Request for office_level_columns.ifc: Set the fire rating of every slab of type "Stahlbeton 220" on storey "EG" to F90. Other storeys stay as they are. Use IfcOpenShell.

First a look at what the model holds.

```python
import ifcopenshell
import ifcopenshell.util.element

model = ifcopenshell.open("office_level_columns.ifc")
print(model.schema)
storey = next(s for s in model.by_type("IfcBuildingStorey") if s.Name == "EG")
slabs = [e for e in ifcopenshell.util.element.get_decomposition(storey) if e.is_a("IfcSlab")]
seen = {}
for e in slabs:
    element_type = ifcopenshell.util.element.get_type(e)
    key = (element_type.Name if element_type != e and element_type else None, ifcopenshell.util.element.get_pset(e, "Pset_SlabCommon", "FireRating"))
    seen[key] = seen.get(key, 0) + 1
for (name, value), count in sorted(seen.items(), key=str):
    print(count, "x", name, "|", value)
```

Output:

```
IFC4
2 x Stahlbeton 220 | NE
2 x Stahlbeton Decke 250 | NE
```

```python
import ifcopenshell
import ifcopenshell.api.pset
import ifcopenshell.util.element

model = ifcopenshell.open("office_level_columns.ifc")

storey = next(s for s in model.by_type("IfcBuildingStorey") if s.Name == "EG")
slabs = [e for e in ifcopenshell.util.element.get_decomposition(storey) if e.is_a("IfcSlab")]

count = 0
for e in slabs:
    element_type = ifcopenshell.util.element.get_type(e)
    if element_type in (None, e) or element_type.Name != "Stahlbeton 220":
        continue
    # add_pset returns the element's existing set when there is one.
    pset = ifcopenshell.api.pset.add_pset(model, product=e, name="Pset_SlabCommon")
    ifcopenshell.api.pset.edit_pset(model, pset=pset, properties={"FireRating": "F90"})
    count += 1

print(count, "slabs updated")

model.write("office_level_columns_updated.ifc")
```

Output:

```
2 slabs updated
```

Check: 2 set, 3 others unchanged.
